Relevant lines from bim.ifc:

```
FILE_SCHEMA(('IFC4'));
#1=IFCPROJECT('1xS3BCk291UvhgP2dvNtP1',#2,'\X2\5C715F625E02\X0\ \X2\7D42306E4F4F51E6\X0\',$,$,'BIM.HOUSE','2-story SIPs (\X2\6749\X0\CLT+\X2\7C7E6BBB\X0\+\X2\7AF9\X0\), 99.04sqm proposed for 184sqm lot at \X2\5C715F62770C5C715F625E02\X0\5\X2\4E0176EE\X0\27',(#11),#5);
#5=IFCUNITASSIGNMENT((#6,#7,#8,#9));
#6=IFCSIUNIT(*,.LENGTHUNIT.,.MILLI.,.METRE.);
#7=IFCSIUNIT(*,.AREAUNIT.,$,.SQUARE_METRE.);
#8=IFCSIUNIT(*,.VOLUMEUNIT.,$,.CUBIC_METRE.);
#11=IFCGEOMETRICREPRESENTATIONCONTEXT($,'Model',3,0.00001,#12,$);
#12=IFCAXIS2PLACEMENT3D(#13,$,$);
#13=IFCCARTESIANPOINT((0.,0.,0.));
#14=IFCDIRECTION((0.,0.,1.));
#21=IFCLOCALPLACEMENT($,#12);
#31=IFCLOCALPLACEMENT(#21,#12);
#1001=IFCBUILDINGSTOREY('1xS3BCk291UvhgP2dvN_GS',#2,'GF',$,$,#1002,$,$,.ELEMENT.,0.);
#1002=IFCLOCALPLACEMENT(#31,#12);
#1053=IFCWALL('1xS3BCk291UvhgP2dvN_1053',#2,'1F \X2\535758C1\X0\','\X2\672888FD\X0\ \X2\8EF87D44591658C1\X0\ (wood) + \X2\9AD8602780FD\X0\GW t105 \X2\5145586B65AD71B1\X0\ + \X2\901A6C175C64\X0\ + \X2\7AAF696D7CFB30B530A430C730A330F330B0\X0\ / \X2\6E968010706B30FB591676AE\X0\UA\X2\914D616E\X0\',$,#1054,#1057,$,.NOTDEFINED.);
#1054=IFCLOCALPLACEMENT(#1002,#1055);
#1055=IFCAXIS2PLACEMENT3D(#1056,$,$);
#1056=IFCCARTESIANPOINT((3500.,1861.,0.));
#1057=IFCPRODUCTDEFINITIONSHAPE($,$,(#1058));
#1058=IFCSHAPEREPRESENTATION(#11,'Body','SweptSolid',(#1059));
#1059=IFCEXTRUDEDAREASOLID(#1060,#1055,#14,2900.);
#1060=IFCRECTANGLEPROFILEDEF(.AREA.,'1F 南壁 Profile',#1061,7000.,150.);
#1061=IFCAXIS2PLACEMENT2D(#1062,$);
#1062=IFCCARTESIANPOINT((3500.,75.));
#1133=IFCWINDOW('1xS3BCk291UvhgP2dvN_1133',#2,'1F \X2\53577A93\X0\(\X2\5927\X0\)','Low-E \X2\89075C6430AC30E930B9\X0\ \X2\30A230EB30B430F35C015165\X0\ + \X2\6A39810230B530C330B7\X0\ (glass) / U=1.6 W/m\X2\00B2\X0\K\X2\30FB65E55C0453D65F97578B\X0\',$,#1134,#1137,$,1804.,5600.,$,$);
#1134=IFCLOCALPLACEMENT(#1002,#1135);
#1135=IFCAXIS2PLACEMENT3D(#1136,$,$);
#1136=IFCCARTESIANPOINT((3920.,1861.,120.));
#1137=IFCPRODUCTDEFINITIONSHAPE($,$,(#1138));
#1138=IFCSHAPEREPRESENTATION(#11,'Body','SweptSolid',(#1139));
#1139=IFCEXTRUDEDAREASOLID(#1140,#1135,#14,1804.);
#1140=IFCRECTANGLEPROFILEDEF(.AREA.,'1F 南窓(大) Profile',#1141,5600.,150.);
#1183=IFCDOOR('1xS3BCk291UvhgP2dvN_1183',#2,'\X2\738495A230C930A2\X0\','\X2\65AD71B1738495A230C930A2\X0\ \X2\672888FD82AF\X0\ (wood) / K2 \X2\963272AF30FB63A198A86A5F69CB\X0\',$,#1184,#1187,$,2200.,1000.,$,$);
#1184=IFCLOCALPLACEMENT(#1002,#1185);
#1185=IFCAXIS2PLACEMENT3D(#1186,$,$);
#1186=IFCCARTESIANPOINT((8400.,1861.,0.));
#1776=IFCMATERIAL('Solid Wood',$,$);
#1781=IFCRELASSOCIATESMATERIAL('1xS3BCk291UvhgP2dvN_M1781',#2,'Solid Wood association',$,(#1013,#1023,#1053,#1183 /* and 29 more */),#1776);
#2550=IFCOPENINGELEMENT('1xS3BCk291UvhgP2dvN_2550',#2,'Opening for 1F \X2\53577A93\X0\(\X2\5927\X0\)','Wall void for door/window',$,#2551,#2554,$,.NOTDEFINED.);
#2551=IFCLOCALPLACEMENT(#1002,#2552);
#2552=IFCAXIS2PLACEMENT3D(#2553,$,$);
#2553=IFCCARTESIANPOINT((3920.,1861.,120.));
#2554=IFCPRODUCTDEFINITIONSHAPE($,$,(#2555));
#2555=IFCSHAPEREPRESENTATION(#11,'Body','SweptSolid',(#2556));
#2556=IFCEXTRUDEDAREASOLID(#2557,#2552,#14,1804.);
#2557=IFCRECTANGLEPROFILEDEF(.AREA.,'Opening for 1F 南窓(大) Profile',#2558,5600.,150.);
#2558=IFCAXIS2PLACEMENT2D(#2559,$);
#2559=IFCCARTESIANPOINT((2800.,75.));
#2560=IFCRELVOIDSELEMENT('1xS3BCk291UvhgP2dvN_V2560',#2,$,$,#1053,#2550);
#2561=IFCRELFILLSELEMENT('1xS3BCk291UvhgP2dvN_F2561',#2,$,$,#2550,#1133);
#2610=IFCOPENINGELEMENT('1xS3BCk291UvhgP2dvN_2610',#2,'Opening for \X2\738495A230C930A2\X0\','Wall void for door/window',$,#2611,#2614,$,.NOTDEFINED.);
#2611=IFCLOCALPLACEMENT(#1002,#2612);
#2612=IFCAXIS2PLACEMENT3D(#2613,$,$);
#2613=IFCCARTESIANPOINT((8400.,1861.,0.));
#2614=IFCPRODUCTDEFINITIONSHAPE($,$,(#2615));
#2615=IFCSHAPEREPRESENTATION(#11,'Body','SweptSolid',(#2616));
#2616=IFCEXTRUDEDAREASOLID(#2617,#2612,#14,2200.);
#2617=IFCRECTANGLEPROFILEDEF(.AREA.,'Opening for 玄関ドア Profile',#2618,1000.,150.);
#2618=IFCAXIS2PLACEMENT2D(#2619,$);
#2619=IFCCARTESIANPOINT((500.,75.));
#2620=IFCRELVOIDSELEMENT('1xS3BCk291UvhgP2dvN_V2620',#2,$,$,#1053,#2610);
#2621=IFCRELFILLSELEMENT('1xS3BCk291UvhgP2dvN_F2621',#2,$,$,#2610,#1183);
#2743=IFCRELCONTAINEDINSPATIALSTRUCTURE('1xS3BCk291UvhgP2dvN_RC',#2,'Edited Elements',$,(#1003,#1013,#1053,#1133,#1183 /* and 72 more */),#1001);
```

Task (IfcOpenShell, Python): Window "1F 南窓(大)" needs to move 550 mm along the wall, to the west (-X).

```python
import ifcopenshell
import ifcopenshell.api.geometry
import ifcopenshell.util.placement

model = ifcopenshell.open("bim.ifc")

window = model.by_guid("1xS3BCk291UvhgP2dvN_1133")
opening = window.FillsVoids[0].RelatingOpeningElement
wall = opening.VoidsElements[0].RelatingBuildingElement

wall_matrix = ifcopenshell.util.placement.get_local_placement(wall.ObjectPlacement)
shift = wall_matrix[:3, 0] * -550.0
before = ifcopenshell.util.placement.get_local_placement(window.ObjectPlacement)[:3, 3].copy()

# The window is not placed relative to its opening, so move both.
for product in (opening, window):
    matrix = ifcopenshell.util.placement.get_local_placement(product.ObjectPlacement)
    matrix[:3, 3] += shift
    ifcopenshell.api.geometry.edit_object_placement(model, product=product, matrix=matrix, is_si=False)

after = ifcopenshell.util.placement.get_local_placement(window.ObjectPlacement)[:3, 3]
print("window moved by", (after - before).round(3) + 0.0)

model.write("bim_updated.ifc")
```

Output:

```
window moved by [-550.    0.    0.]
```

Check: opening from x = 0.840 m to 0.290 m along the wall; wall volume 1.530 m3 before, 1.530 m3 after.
